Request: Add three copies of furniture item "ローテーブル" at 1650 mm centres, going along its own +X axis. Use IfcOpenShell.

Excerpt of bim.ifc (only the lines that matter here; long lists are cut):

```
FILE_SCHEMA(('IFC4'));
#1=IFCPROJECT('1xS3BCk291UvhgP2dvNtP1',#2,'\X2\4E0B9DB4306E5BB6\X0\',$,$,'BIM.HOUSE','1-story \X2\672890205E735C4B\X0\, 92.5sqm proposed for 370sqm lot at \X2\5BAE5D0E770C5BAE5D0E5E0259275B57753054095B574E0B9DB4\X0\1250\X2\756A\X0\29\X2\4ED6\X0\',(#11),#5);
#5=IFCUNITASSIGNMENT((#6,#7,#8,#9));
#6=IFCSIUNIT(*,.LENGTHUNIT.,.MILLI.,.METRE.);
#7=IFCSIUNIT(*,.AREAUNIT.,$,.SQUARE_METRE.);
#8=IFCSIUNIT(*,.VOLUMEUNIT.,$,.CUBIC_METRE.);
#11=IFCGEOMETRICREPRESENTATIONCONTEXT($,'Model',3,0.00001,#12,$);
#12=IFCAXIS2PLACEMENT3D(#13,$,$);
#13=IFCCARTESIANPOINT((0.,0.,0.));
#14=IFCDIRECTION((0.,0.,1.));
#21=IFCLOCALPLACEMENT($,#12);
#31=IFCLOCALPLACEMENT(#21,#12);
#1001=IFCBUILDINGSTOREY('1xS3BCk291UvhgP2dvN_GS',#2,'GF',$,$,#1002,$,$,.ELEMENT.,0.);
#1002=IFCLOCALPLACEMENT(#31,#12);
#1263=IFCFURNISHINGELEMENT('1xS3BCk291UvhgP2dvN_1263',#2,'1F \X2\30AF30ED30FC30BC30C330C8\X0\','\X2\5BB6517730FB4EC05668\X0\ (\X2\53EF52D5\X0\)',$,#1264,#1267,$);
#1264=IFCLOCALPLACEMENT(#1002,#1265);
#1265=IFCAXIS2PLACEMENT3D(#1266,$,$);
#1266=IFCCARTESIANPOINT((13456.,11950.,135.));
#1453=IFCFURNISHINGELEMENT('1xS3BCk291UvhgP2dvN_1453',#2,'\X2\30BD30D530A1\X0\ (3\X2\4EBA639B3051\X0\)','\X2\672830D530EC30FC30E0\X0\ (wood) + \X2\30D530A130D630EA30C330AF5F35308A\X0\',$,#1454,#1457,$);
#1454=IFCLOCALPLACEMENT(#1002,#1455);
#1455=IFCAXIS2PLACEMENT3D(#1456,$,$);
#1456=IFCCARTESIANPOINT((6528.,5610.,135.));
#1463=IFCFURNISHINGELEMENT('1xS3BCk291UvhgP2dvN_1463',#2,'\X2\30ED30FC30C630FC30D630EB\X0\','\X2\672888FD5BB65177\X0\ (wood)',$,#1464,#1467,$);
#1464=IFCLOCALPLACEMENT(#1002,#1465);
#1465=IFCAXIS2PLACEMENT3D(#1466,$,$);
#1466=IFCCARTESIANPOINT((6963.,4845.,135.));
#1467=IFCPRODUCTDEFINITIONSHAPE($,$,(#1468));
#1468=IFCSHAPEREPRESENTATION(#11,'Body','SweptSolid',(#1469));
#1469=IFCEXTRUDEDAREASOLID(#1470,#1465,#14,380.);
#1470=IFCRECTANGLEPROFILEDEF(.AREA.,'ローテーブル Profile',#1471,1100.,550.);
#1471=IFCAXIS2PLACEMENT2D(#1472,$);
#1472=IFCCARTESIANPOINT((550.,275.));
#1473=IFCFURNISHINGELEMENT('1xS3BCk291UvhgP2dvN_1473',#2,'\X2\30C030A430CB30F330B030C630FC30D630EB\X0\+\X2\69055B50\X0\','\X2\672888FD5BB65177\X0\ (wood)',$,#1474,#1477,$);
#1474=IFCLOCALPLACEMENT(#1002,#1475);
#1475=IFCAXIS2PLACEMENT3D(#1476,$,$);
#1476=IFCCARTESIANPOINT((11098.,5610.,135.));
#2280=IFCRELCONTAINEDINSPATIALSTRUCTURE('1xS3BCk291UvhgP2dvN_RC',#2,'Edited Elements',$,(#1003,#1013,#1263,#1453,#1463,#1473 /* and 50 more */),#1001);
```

```python
import ifcopenshell
import ifcopenshell.api.geometry
import ifcopenshell.api.root
import ifcopenshell.util.element
import ifcopenshell.util.placement
import ifcopenshell.util.unit

model = ifcopenshell.open("bim.ifc")
unit_scale = ifcopenshell.util.unit.calculate_unit_scale(model)


def reuse_history(source, copy):
    """copy_class also copies each property set's owner history, people and application; keep the originals."""
    for rel in copy.IsDefinedBy:
        if rel.is_a("IfcRelDefinesByProperties") and (history := rel.RelatingPropertyDefinition.OwnerHistory):
            rel.RelatingPropertyDefinition.OwnerHistory = source.OwnerHistory
            ifcopenshell.util.element.remove_deep2(model, history)


source = model.by_id(1463)
base = ifcopenshell.util.placement.get_local_placement(source.ObjectPlacement)
step = base[:3, 0] * 1.65 / unit_scale

for i in range(1, 4):
    copy = ifcopenshell.api.root.copy_class(model, product=source)
    copy.Representation = ifcopenshell.util.element.copy_deep(
        model, source.Representation, exclude=["IfcGeometricRepresentationContext", "IfcRepresentationMap"]
    )
    reuse_history(source, copy)
    matrix = base.copy()
    matrix[:3, 3] += i * step
    print("added at", matrix[:3, 3].round(3) + 0.0)
    ifcopenshell.api.geometry.edit_object_placement(model, product=copy, matrix=matrix, is_si=False)

model.write("bim-out.ifc")
```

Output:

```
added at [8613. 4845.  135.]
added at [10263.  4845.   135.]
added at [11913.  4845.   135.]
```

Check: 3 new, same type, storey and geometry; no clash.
